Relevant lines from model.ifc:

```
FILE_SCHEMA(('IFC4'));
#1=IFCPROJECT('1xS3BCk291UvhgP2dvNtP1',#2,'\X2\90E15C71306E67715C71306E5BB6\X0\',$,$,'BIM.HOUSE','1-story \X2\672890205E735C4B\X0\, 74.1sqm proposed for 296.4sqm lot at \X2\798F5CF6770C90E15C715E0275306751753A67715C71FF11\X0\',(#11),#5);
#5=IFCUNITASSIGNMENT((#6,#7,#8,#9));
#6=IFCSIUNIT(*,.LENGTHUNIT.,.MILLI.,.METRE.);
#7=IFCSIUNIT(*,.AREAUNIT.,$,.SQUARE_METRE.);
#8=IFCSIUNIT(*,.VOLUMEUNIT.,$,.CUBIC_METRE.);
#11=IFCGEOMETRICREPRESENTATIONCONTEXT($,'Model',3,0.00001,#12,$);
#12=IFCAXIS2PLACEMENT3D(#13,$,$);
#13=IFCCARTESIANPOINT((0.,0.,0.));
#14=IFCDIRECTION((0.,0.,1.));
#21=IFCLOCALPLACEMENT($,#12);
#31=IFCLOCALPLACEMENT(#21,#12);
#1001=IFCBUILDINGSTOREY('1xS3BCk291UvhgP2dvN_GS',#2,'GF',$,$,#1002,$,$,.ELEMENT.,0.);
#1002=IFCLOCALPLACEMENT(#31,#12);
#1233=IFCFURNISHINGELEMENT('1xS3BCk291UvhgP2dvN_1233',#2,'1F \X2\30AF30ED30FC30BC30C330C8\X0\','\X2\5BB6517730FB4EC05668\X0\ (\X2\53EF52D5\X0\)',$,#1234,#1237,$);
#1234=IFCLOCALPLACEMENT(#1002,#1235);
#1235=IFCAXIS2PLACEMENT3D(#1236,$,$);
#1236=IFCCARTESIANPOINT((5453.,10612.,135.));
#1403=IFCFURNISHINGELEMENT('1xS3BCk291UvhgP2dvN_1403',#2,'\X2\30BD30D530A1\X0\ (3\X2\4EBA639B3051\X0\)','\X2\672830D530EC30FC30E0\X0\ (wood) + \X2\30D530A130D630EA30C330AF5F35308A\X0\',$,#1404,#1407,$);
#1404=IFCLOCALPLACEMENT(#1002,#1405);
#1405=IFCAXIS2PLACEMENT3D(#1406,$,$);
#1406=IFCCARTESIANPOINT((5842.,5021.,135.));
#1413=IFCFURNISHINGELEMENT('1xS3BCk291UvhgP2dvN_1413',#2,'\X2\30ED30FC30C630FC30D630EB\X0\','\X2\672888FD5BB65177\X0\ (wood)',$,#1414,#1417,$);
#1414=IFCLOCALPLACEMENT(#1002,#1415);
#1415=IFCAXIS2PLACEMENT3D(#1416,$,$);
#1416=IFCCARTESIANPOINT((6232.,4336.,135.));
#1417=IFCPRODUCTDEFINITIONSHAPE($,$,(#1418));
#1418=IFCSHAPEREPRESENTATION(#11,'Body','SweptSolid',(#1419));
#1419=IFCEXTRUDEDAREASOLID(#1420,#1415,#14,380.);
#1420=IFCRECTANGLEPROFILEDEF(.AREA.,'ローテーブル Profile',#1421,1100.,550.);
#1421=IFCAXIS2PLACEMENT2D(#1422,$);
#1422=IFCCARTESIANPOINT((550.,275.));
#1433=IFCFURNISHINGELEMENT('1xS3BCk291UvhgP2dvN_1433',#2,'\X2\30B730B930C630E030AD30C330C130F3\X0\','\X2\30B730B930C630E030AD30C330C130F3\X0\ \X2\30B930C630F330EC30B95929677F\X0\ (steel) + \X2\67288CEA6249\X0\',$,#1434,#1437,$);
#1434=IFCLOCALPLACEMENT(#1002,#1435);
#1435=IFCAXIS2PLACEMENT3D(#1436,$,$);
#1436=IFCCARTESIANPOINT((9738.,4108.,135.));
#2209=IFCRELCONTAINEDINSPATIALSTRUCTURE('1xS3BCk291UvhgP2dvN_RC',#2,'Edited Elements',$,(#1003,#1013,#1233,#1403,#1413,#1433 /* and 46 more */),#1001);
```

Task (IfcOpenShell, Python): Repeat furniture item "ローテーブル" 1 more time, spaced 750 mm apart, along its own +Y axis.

```python
import ifcopenshell
import ifcopenshell.api.geometry
import ifcopenshell.api.root
import ifcopenshell.util.element
import ifcopenshell.util.placement
import ifcopenshell.util.unit

model = ifcopenshell.open("model.ifc")
unit_scale = ifcopenshell.util.unit.calculate_unit_scale(model)


def reuse_history(source, copy):
    """copy_class also copies each property set's owner history, people and application; keep the originals."""
    for rel in copy.IsDefinedBy:
        if rel.is_a("IfcRelDefinesByProperties") and (history := rel.RelatingPropertyDefinition.OwnerHistory):
            rel.RelatingPropertyDefinition.OwnerHistory = source.OwnerHistory
            ifcopenshell.util.element.remove_deep2(model, history)


source = model.by_guid("1xS3BCk291UvhgP2dvN_1413")
base = ifcopenshell.util.placement.get_local_placement(source.ObjectPlacement)
step = base[:3, 1] * 0.75 / unit_scale

for i in range(1, 2):
    copy = ifcopenshell.api.root.copy_class(model, product=source)
    copy.Representation = ifcopenshell.util.element.copy_deep(
        model, source.Representation, exclude=["IfcGeometricRepresentationContext", "IfcRepresentationMap"]
    )
    reuse_history(source, copy)
    matrix = base.copy()
    matrix[:3, 3] += i * step
    print("added at", matrix[:3, 3].round(3) + 0.0)
    ifcopenshell.api.geometry.edit_object_placement(model, product=copy, matrix=matrix, is_si=False)

model.write("model_rev.ifc")
```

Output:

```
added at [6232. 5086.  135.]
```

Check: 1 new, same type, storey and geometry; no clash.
